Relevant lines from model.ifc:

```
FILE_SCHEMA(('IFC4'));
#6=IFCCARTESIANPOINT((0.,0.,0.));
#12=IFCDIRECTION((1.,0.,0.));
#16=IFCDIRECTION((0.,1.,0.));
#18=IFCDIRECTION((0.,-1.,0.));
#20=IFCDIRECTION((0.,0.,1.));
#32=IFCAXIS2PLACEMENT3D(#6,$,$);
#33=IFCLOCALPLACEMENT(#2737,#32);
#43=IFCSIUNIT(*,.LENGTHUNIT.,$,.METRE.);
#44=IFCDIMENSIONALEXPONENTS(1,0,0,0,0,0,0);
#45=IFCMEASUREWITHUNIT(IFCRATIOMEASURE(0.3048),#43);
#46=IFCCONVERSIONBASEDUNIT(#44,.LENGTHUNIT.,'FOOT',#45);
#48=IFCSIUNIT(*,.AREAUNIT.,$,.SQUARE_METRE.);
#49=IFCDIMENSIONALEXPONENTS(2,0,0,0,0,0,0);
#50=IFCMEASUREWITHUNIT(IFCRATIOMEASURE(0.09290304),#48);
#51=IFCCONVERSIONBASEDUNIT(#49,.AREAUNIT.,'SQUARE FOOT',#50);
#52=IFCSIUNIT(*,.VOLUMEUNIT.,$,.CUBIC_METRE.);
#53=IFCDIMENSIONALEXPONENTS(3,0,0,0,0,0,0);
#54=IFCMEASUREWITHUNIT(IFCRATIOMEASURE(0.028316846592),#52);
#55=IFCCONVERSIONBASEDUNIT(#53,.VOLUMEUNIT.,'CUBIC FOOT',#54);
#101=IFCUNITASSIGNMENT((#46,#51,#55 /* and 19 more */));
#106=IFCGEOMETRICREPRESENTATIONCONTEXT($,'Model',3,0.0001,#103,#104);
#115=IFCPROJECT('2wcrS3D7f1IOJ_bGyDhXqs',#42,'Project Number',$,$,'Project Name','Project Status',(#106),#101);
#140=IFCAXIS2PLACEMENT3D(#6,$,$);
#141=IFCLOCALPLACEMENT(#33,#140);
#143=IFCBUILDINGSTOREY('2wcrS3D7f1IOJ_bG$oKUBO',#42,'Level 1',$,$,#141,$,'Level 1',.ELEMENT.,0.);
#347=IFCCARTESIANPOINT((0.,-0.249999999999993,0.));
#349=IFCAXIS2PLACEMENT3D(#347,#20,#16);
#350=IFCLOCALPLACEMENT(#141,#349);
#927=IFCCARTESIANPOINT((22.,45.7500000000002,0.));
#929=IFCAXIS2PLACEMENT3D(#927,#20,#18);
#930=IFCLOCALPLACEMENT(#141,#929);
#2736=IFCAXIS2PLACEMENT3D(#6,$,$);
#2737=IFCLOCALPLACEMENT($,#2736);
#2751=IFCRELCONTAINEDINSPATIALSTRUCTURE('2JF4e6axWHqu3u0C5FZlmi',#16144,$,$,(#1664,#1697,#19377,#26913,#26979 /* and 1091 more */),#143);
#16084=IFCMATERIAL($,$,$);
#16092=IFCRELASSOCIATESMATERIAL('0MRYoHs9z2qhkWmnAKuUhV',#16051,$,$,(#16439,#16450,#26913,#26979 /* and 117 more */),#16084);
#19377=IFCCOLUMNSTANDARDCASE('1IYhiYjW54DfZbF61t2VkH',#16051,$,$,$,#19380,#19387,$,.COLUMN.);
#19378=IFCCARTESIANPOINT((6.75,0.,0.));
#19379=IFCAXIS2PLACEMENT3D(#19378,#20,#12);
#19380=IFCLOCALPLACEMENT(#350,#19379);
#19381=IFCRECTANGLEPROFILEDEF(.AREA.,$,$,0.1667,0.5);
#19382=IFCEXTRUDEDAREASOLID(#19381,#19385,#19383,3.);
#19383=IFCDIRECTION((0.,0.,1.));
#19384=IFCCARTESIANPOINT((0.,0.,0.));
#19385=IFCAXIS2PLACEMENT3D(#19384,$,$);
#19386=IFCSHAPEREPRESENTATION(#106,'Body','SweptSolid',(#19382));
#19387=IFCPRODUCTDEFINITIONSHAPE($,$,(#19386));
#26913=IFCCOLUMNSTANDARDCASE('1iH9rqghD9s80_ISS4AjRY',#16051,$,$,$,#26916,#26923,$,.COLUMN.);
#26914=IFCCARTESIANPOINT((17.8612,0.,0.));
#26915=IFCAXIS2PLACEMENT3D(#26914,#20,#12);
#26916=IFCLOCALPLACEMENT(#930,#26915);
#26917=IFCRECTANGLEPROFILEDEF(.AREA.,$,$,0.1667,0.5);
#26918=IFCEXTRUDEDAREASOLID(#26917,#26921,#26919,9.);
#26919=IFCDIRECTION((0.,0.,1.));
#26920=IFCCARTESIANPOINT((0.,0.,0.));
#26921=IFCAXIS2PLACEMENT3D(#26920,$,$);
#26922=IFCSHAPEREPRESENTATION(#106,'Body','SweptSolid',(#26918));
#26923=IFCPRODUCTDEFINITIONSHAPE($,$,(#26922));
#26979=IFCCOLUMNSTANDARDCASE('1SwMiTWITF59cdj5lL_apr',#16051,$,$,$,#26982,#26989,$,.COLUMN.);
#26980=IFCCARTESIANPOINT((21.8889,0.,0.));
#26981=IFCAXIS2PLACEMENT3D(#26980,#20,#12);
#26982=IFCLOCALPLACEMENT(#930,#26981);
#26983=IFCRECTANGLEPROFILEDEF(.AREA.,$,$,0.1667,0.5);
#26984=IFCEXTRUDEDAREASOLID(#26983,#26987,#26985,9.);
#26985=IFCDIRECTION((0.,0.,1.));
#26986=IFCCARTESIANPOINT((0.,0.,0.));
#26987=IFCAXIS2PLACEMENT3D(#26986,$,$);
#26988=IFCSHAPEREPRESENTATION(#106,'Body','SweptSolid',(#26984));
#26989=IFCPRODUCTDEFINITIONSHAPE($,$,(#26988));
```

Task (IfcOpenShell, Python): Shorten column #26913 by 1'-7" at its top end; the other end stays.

```python
import ifcopenshell
import ifcopenshell.util.unit

model = ifcopenshell.open("model.ifc")
unit_scale = ifcopenshell.util.unit.calculate_unit_scale(model)

member = model.by_id(26913)
change = -19 * 0.0254 / unit_scale

# The extrusion runs towards the end named, so only its depth changes.
body = next(r for r in member.Representation.Representations if r.RepresentationIdentifier == "Body")
solid = body.Items[0]
old_length = solid.Depth
solid.Depth += change

print(f"length {old_length:g} -> {solid.Depth:g}")

model.write("model_rev.ifc")
```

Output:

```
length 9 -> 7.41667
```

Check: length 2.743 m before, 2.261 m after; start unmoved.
